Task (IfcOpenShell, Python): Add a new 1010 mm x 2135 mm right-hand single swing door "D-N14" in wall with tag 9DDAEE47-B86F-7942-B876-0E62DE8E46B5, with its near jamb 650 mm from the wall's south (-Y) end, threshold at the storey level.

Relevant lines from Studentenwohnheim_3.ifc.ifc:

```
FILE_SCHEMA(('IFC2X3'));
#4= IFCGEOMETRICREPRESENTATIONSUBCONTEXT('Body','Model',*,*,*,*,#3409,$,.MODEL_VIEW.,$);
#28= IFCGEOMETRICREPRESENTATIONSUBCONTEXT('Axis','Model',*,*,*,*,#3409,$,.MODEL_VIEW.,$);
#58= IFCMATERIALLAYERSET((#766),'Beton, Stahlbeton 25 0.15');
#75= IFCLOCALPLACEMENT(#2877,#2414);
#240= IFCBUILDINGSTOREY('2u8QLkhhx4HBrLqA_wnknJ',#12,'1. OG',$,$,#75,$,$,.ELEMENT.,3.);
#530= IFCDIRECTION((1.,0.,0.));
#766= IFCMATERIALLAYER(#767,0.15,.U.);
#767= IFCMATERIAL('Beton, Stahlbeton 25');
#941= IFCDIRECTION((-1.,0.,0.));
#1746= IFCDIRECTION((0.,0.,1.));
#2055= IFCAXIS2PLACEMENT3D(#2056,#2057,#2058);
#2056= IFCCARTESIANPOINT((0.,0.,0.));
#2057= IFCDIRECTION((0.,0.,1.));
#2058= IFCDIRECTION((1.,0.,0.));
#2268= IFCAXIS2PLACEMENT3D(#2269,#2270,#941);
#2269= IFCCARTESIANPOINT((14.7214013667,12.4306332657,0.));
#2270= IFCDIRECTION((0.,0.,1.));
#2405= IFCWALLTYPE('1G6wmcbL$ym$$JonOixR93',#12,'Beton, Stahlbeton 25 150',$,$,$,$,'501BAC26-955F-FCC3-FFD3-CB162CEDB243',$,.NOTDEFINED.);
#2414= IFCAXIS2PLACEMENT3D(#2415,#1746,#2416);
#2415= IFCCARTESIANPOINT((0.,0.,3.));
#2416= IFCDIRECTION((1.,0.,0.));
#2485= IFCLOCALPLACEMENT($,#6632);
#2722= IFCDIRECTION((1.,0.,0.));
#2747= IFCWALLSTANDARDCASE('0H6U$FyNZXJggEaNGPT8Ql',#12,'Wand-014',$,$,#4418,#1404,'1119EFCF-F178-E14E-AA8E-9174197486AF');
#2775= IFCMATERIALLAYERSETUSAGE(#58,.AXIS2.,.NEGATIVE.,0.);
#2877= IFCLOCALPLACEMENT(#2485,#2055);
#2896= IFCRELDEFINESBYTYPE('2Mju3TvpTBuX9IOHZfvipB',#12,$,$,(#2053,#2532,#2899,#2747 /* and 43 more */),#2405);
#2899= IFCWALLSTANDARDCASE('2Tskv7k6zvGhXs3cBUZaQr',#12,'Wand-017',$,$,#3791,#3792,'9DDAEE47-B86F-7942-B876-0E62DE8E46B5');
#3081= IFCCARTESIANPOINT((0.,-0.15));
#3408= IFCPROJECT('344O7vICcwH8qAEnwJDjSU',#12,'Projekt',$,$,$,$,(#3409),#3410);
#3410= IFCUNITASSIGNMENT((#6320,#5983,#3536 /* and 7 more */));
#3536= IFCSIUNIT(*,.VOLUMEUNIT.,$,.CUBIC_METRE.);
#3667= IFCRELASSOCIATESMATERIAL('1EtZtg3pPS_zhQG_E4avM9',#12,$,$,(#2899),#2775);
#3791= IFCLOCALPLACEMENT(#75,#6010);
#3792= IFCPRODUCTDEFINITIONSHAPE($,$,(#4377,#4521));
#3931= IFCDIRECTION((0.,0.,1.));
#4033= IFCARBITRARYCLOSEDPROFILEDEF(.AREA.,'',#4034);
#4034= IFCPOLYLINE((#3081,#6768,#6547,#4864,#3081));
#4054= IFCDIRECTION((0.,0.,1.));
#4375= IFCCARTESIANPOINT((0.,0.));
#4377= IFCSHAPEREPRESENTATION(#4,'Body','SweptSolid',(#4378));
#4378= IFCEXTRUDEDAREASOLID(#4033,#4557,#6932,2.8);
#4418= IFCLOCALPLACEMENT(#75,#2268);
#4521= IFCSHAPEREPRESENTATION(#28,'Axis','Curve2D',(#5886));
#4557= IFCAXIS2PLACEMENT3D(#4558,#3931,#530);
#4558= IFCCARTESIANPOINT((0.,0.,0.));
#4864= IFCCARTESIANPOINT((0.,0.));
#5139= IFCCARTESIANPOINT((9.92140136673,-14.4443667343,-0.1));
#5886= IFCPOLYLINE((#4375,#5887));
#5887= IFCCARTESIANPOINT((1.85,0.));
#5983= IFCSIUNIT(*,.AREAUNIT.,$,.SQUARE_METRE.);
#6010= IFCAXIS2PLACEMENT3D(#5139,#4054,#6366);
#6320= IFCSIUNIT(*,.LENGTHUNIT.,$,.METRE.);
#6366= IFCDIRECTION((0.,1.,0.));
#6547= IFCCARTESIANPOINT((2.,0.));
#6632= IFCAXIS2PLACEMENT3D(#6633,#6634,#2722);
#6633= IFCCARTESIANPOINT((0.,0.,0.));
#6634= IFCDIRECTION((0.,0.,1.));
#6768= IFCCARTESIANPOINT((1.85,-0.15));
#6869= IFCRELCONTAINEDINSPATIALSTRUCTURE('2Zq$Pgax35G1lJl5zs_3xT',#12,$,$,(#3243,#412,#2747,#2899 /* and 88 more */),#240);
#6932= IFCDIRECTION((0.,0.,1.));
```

```python
import numpy as np
import ifcopenshell
import ifcopenshell.api.feature
import ifcopenshell.api.geometry
import ifcopenshell.api.root
import ifcopenshell.api.spatial
import ifcopenshell.api.type
import ifcopenshell.geom
import ifcopenshell.util.element
import ifcopenshell.util.placement
import ifcopenshell.util.representation
import ifcopenshell.util.shape
import ifcopenshell.util.unit

model = ifcopenshell.open("Studentenwohnheim_3.ifc.ifc")
unit_scale = ifcopenshell.util.unit.calculate_unit_scale(model)
settings = ifcopenshell.geom.settings()


def volume(element):
    """Net volume in cubic metres, openings subtracted."""
    shape = ifcopenshell.geom.create_shape(settings, element)
    return ifcopenshell.util.shape.get_volume(shape.geometry)


wall = model.by_guid("2Tskv7k6zvGhXs3cBUZaQr")
storey = ifcopenshell.util.element.get_container(wall, ifc_class="IfcBuildingStorey")
context = ifcopenshell.util.representation.get_context(model, "Model", "Body", "MODEL_VIEW")
before = volume(wall)

width, height, from_end, sill = 1.01, 2.135, 0.65, 0.0  # metres

# The wall runs along its own X axis, and the end named is its -X end.
wall_shape = ifcopenshell.geom.create_shape(settings, wall)
x, y, z = ifcopenshell.util.shape.get_vertices(wall_shape.geometry).T
start = x.min() + from_end
face, thickness = float(y.min()), float(y.max() - y.min())
wall_matrix = ifcopenshell.util.placement.get_local_placement(wall.ObjectPlacement)
level = ifcopenshell.util.placement.get_local_placement(storey.ObjectPlacement)[2, 3]


def in_wall(x, y):
    """Placement at x, y metres in the wall's axes, at sill height."""
    matrix = wall_matrix.copy()
    matrix[:, 3] = wall_matrix @ np.array([x / unit_scale, y / unit_scale, 0.0, 1.0])
    matrix[2, 3] = level + sill / unit_scale
    return matrix


# Opening: a box that overshoots both wall faces by 50 mm.
opening = ifcopenshell.api.root.create_entity(model, ifc_class="IfcOpeningElement")
box = ifcopenshell.api.geometry.add_wall_representation(
    model, context=context, length=width, height=height, thickness=thickness + 0.1
)
ifcopenshell.api.geometry.assign_representation(model, product=opening, representation=box)
ifcopenshell.api.geometry.edit_object_placement(model, product=opening, matrix=in_wall(start, face - 0.05), is_si=False)
ifcopenshell.api.feature.add_feature(model, feature=opening, element=wall)

door = ifcopenshell.api.root.create_entity(model, ifc_class="IfcDoor", name="D-N14")
door.OverallWidth, door.OverallHeight = width / unit_scale, height / unit_scale
body = ifcopenshell.api.geometry.add_door_representation(
    model,
    context=context,
    overall_width=door.OverallWidth,
    overall_height=door.OverallHeight,
    operation_type="SINGLE_SWING_RIGHT",
    lining_properties={"LiningDepth": thickness / unit_scale, "ThresholdDepth": thickness / unit_scale},
)
ifcopenshell.api.geometry.assign_representation(model, product=door, representation=body)
ifcopenshell.api.spatial.assign_container(model, products=[door], relating_structure=storey)
fills = ifcopenshell.api.feature.add_filling(model, opening=opening, element=door)
fills.OwnerHistory = door.OwnerHistory  # required in IFC2X3

# IFC2X3 keeps the operation on the door style.
style = ifcopenshell.api.root.create_entity(model, ifc_class="IfcDoorStyle", name="D-N14")
style.OperationType, style.ConstructionType = "SINGLE_SWING_RIGHT", "NOTDEFINED"
style.ParameterTakesPrecedence = style.Sizeable = False
ifcopenshell.api.type.assign_type(model, related_objects=[door], relating_type=style)

# The lining spans the wall, so the door starts at the wall face.
ifcopenshell.api.geometry.edit_object_placement(model, product=door, matrix=in_wall(start, face), is_si=False)

after = volume(wall)

print(f"wall volume {before:.3f} -> {after:.3f} m3")

model.write("Studentenwohnheim_3.ifc_updated.ifc")
```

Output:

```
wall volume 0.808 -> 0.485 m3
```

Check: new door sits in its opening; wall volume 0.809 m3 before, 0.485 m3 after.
